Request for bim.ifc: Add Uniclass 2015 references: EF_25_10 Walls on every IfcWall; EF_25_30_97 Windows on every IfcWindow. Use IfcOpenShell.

First a look at what the model holds.

```python
import ifcopenshell

model = ifcopenshell.open("bim.ifc")
print(model.schema)
print("classifications:", [c.Name for c in model.by_type("IfcClassification")])
for ifc_class in ("IfcDoor", "IfcRoof", "IfcStair", "IfcWall", "IfcWindow"):
    print(ifc_class, len(model.by_type(ifc_class)))
```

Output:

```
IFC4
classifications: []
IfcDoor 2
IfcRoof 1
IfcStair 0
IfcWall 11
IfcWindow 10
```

```python
import ifcopenshell
import ifcopenshell.api.classification

model = ifcopenshell.open("bim.ifc")

system = ifcopenshell.api.classification.add_classification(model, classification="Uniclass 2015")

codes = {
    "IfcWall": ("EF_25_10", "Walls"),
    "IfcWindow": ("EF_25_30_97", "Windows"),
}
for ifc_class, (code, name) in codes.items():
    products = model.by_type(ifc_class)
    ifcopenshell.api.classification.add_reference(
        model, products=products, classification=system, identification=code, name=name
    )
    print(code, len(products))

model.write("bim_v2.ifc")
```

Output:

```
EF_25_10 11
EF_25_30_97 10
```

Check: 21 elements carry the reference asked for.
